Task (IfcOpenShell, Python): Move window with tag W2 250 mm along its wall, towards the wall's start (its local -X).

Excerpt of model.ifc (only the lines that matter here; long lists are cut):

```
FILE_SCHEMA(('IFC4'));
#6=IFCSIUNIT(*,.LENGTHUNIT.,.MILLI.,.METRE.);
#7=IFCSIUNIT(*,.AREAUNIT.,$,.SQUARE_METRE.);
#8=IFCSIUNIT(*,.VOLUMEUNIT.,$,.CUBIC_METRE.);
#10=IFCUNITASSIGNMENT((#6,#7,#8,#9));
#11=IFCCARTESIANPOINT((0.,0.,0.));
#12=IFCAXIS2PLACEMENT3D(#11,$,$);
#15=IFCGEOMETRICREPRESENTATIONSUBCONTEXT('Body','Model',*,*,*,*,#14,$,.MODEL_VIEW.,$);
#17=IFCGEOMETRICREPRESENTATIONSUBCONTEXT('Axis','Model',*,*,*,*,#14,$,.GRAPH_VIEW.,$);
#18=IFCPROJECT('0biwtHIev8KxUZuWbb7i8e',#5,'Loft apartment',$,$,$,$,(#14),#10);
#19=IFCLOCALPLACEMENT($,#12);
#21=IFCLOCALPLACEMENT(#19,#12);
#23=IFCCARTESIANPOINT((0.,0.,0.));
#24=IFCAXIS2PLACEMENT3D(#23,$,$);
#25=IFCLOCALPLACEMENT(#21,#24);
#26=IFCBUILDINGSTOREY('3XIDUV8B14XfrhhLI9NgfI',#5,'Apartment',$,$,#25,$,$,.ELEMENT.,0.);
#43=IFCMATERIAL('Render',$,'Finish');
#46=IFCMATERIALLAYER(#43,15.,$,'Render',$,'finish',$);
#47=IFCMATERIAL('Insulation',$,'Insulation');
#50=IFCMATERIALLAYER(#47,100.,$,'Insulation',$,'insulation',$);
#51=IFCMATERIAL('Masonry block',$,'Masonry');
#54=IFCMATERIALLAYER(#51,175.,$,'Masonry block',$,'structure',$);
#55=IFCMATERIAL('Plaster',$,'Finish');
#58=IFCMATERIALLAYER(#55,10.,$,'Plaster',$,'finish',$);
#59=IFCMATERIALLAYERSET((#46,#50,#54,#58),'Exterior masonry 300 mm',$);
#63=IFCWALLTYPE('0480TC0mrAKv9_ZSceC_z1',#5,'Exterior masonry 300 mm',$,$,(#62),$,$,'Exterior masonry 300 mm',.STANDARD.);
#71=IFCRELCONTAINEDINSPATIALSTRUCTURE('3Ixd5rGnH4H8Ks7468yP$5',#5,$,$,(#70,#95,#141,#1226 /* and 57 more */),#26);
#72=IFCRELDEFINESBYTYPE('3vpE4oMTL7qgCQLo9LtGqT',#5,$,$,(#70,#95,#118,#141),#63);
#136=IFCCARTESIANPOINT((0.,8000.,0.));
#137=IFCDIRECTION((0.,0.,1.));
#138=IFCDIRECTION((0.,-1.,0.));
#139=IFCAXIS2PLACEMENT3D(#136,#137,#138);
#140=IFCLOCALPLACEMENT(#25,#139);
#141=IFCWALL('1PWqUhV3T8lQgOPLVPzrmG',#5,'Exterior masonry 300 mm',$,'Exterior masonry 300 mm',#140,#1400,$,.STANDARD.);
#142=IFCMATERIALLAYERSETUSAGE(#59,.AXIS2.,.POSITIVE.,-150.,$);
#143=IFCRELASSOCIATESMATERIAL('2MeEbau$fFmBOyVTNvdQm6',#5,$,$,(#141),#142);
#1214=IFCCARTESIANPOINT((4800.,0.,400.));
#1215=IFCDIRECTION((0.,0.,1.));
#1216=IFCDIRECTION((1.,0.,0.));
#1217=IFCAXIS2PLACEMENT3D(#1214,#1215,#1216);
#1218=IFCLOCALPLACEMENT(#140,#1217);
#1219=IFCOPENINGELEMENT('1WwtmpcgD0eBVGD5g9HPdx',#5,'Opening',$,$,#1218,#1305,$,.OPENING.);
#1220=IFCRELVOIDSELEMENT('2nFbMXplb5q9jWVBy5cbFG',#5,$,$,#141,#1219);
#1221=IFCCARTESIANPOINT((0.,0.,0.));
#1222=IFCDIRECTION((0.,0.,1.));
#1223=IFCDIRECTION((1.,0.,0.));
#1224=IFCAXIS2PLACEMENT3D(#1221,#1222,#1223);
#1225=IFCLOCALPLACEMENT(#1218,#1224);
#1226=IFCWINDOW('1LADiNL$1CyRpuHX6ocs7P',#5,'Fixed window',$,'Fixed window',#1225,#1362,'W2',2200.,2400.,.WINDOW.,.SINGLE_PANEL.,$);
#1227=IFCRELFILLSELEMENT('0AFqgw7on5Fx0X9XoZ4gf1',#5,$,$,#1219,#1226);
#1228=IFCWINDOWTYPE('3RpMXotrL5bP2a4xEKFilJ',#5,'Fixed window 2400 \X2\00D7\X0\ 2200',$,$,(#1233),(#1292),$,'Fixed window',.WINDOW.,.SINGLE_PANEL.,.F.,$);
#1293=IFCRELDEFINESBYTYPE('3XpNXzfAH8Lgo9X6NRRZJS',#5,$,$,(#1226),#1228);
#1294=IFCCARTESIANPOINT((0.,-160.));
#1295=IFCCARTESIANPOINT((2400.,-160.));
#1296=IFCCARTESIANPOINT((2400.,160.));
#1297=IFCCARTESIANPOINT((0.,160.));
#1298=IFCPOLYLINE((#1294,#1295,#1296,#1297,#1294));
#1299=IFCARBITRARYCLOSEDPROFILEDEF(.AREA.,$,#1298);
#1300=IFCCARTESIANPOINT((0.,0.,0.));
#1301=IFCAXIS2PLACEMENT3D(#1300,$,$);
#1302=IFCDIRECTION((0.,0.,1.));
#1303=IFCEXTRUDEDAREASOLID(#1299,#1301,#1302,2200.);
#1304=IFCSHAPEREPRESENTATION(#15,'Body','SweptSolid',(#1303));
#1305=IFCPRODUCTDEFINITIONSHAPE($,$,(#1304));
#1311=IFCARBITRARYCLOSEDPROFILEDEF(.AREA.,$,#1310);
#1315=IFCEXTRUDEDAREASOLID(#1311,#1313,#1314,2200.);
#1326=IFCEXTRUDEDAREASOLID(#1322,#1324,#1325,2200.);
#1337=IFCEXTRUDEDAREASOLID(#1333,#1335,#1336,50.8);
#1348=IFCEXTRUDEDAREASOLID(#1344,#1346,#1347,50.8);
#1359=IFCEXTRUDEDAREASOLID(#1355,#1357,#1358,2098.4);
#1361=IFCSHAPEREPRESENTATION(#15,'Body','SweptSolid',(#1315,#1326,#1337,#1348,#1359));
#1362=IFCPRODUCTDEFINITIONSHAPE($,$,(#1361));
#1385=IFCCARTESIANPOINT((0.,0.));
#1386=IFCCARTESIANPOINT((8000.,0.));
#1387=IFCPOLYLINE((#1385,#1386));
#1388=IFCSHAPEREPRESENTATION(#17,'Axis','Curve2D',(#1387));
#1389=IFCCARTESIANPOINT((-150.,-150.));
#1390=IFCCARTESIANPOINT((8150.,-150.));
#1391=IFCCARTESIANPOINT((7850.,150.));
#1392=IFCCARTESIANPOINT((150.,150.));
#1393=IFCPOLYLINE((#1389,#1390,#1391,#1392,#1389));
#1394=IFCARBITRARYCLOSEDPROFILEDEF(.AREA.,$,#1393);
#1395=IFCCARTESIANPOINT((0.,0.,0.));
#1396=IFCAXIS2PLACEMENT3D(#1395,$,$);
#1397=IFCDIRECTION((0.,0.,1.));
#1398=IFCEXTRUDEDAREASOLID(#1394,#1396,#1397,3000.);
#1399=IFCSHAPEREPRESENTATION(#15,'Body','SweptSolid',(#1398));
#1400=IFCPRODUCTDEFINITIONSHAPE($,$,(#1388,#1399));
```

```python
import ifcopenshell
import ifcopenshell.api.geometry
import ifcopenshell.util.placement
import ifcopenshell.util.unit

model = ifcopenshell.open("model.ifc")
unit_scale = ifcopenshell.util.unit.calculate_unit_scale(model)

window = model.by_id(1226)
opening = window.FillsVoids[0].RelatingOpeningElement
wall = opening.VoidsElements[0].RelatingBuildingElement

wall_matrix = ifcopenshell.util.placement.get_local_placement(wall.ObjectPlacement)
shift = wall_matrix[:3, 0] * -0.25 / unit_scale
before = ifcopenshell.util.placement.get_local_placement(window.ObjectPlacement)[:3, 3].copy()

# The window is placed relative to its opening, so it follows when the opening moves.
matrix = ifcopenshell.util.placement.get_local_placement(opening.ObjectPlacement)
matrix[:3, 3] += shift
ifcopenshell.api.geometry.edit_object_placement(
    model, product=opening, matrix=matrix, is_si=False, should_transform_children=True
)

after = ifcopenshell.util.placement.get_local_placement(window.ObjectPlacement)[:3, 3]
print("window moved by", (after - before).round(3) + 0.0)

model.write("model_v2.ifc")
```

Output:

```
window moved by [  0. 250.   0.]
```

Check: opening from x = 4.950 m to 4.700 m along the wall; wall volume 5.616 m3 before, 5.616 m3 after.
